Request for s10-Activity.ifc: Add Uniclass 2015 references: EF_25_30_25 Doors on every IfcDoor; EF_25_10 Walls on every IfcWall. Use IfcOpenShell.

First a look at what the model holds.

```python
import ifcopenshell

model = ifcopenshell.open("s10-Activity.ifc")
print(model.schema)
print("classifications:", [c.Name for c in model.by_type("IfcClassification")])
for ifc_class in ("IfcDoor", "IfcRoof", "IfcStair", "IfcWall", "IfcWindow"):
    print(ifc_class, len(model.by_type(ifc_class)))
```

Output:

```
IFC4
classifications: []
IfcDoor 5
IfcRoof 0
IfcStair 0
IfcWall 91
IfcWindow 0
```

```python
import ifcopenshell
import ifcopenshell.api.classification

model = ifcopenshell.open("s10-Activity.ifc")

system = ifcopenshell.api.classification.add_classification(model, classification="Uniclass 2015")

codes = {
    "IfcDoor": ("EF_25_30_25", "Doors"),
    "IfcWall": ("EF_25_10", "Walls"),
}
for ifc_class, (code, name) in codes.items():
    products = model.by_type(ifc_class)
    ifcopenshell.api.classification.add_reference(
        model, products=products, classification=system, identification=code, name=name
    )
    print(code, len(products))

model.write("s10-Activity_updated.ifc")
```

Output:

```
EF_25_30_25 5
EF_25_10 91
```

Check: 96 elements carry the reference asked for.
